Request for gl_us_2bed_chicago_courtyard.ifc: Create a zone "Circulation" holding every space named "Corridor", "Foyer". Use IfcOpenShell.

First a look at what the model holds.

```python
import ifcopenshell

model = ifcopenshell.open("gl_us_2bed_chicago_courtyard.ifc")
print(model.schema)
seen = {}
for space in model.by_type("IfcSpace"):
    seen[space.LongName] = seen.get(space.LongName, 0) + 1
for name, count in sorted(seen.items(), key=str):
    print(count, "x", name)
print("zones:", [z.Name for z in model.by_type("IfcZone")][:20])
```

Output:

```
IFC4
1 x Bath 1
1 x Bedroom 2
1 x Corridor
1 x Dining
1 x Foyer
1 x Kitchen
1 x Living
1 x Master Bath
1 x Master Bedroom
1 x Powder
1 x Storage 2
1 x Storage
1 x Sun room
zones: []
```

```python
import ifcopenshell
import ifcopenshell.api.group
import ifcopenshell.api.root

model = ifcopenshell.open("gl_us_2bed_chicago_courtyard.ifc")

names = {"Corridor", "Foyer"}
spaces = [s for s in model.by_type("IfcSpace") if s.LongName in names]

zone = ifcopenshell.api.root.create_entity(model, ifc_class="IfcZone", name="Circulation")
ifcopenshell.api.group.assign_group(model, products=spaces, group=zone)
print(len(spaces), "spaces in", zone.Name)

model.write("gl_us_2bed_chicago_courtyard_rev.ifc")
```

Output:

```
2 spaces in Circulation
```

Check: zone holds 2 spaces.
